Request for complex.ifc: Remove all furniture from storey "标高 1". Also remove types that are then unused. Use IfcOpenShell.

First a look at what the model holds.

```python
import ifcopenshell
import ifcopenshell.util.element

model = ifcopenshell.open("complex.ifc")
print(model.schema)
storey = next(s for s in model.by_type("IfcBuildingStorey") if s.Name == "标高 1")
furniture = [e for e in ifcopenshell.util.element.get_decomposition(storey) if e.is_a("IfcFurnishingElement")]
seen = {}
for e in furniture:
    element_type = ifcopenshell.util.element.get_type(e)
    name = element_type.Name if element_type not in (None, e) else None
    seen[name] = seen.get(name, 0) + 1
for name, count in sorted(seen.items(), key=str):
    print(count, "x", name)
```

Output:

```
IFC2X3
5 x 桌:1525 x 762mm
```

```python
import ifcopenshell
import ifcopenshell.api.root
import ifcopenshell.util.element

model = ifcopenshell.open("complex.ifc")

storey = next(s for s in model.by_type("IfcBuildingStorey") if s.Name == "标高 1")
furniture = [e for e in ifcopenshell.util.element.get_decomposition(storey) if e.is_a("IfcFurnishingElement")]
types = {ifcopenshell.util.element.get_type(e) for e in furniture} - {None, *furniture}

for e in furniture:
    ifcopenshell.api.root.remove_product(model, product=e)
print(len(furniture), "removed")

unused = [t for t in types if not ifcopenshell.util.element.get_types(t)]
for t in unused:
    ifcopenshell.api.root.remove_product(model, product=t)
print(len(unused), "unused types removed")

model.write("complex-out.ifc")
```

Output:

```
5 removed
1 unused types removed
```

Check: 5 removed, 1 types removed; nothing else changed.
